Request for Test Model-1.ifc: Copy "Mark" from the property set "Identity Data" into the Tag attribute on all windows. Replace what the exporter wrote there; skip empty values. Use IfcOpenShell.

First a look at what the model holds.

```python
import ifcopenshell
import ifcopenshell.util.element

model = ifcopenshell.open("Test Model-1.ifc")
print(model.schema)
windows = model.by_type("IfcWindow")
print(len(windows), "windows")
for e in windows[:8]:
    source = ifcopenshell.util.element.get_pset(e, "Identity Data", "Mark")
    target = e.Tag
    print(e.id(), repr(source), repr(target), sep=" | ")
```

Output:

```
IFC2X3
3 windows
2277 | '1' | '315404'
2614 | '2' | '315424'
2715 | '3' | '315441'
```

```python
import ifcopenshell
import ifcopenshell.util.element

model = ifcopenshell.open("Test Model-1.ifc")

count = 0
for e in model.by_type("IfcWindow"):
    value = ifcopenshell.util.element.get_pset(e, "Identity Data", "Mark")
    current = e.Tag
    if not value or not value.strip() or current == value:
        continue
    e.Tag = value
    count += 1

print(count, "windows updated")

model.write("Test Model-1_v2.ifc")
```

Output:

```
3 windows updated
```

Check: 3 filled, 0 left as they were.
